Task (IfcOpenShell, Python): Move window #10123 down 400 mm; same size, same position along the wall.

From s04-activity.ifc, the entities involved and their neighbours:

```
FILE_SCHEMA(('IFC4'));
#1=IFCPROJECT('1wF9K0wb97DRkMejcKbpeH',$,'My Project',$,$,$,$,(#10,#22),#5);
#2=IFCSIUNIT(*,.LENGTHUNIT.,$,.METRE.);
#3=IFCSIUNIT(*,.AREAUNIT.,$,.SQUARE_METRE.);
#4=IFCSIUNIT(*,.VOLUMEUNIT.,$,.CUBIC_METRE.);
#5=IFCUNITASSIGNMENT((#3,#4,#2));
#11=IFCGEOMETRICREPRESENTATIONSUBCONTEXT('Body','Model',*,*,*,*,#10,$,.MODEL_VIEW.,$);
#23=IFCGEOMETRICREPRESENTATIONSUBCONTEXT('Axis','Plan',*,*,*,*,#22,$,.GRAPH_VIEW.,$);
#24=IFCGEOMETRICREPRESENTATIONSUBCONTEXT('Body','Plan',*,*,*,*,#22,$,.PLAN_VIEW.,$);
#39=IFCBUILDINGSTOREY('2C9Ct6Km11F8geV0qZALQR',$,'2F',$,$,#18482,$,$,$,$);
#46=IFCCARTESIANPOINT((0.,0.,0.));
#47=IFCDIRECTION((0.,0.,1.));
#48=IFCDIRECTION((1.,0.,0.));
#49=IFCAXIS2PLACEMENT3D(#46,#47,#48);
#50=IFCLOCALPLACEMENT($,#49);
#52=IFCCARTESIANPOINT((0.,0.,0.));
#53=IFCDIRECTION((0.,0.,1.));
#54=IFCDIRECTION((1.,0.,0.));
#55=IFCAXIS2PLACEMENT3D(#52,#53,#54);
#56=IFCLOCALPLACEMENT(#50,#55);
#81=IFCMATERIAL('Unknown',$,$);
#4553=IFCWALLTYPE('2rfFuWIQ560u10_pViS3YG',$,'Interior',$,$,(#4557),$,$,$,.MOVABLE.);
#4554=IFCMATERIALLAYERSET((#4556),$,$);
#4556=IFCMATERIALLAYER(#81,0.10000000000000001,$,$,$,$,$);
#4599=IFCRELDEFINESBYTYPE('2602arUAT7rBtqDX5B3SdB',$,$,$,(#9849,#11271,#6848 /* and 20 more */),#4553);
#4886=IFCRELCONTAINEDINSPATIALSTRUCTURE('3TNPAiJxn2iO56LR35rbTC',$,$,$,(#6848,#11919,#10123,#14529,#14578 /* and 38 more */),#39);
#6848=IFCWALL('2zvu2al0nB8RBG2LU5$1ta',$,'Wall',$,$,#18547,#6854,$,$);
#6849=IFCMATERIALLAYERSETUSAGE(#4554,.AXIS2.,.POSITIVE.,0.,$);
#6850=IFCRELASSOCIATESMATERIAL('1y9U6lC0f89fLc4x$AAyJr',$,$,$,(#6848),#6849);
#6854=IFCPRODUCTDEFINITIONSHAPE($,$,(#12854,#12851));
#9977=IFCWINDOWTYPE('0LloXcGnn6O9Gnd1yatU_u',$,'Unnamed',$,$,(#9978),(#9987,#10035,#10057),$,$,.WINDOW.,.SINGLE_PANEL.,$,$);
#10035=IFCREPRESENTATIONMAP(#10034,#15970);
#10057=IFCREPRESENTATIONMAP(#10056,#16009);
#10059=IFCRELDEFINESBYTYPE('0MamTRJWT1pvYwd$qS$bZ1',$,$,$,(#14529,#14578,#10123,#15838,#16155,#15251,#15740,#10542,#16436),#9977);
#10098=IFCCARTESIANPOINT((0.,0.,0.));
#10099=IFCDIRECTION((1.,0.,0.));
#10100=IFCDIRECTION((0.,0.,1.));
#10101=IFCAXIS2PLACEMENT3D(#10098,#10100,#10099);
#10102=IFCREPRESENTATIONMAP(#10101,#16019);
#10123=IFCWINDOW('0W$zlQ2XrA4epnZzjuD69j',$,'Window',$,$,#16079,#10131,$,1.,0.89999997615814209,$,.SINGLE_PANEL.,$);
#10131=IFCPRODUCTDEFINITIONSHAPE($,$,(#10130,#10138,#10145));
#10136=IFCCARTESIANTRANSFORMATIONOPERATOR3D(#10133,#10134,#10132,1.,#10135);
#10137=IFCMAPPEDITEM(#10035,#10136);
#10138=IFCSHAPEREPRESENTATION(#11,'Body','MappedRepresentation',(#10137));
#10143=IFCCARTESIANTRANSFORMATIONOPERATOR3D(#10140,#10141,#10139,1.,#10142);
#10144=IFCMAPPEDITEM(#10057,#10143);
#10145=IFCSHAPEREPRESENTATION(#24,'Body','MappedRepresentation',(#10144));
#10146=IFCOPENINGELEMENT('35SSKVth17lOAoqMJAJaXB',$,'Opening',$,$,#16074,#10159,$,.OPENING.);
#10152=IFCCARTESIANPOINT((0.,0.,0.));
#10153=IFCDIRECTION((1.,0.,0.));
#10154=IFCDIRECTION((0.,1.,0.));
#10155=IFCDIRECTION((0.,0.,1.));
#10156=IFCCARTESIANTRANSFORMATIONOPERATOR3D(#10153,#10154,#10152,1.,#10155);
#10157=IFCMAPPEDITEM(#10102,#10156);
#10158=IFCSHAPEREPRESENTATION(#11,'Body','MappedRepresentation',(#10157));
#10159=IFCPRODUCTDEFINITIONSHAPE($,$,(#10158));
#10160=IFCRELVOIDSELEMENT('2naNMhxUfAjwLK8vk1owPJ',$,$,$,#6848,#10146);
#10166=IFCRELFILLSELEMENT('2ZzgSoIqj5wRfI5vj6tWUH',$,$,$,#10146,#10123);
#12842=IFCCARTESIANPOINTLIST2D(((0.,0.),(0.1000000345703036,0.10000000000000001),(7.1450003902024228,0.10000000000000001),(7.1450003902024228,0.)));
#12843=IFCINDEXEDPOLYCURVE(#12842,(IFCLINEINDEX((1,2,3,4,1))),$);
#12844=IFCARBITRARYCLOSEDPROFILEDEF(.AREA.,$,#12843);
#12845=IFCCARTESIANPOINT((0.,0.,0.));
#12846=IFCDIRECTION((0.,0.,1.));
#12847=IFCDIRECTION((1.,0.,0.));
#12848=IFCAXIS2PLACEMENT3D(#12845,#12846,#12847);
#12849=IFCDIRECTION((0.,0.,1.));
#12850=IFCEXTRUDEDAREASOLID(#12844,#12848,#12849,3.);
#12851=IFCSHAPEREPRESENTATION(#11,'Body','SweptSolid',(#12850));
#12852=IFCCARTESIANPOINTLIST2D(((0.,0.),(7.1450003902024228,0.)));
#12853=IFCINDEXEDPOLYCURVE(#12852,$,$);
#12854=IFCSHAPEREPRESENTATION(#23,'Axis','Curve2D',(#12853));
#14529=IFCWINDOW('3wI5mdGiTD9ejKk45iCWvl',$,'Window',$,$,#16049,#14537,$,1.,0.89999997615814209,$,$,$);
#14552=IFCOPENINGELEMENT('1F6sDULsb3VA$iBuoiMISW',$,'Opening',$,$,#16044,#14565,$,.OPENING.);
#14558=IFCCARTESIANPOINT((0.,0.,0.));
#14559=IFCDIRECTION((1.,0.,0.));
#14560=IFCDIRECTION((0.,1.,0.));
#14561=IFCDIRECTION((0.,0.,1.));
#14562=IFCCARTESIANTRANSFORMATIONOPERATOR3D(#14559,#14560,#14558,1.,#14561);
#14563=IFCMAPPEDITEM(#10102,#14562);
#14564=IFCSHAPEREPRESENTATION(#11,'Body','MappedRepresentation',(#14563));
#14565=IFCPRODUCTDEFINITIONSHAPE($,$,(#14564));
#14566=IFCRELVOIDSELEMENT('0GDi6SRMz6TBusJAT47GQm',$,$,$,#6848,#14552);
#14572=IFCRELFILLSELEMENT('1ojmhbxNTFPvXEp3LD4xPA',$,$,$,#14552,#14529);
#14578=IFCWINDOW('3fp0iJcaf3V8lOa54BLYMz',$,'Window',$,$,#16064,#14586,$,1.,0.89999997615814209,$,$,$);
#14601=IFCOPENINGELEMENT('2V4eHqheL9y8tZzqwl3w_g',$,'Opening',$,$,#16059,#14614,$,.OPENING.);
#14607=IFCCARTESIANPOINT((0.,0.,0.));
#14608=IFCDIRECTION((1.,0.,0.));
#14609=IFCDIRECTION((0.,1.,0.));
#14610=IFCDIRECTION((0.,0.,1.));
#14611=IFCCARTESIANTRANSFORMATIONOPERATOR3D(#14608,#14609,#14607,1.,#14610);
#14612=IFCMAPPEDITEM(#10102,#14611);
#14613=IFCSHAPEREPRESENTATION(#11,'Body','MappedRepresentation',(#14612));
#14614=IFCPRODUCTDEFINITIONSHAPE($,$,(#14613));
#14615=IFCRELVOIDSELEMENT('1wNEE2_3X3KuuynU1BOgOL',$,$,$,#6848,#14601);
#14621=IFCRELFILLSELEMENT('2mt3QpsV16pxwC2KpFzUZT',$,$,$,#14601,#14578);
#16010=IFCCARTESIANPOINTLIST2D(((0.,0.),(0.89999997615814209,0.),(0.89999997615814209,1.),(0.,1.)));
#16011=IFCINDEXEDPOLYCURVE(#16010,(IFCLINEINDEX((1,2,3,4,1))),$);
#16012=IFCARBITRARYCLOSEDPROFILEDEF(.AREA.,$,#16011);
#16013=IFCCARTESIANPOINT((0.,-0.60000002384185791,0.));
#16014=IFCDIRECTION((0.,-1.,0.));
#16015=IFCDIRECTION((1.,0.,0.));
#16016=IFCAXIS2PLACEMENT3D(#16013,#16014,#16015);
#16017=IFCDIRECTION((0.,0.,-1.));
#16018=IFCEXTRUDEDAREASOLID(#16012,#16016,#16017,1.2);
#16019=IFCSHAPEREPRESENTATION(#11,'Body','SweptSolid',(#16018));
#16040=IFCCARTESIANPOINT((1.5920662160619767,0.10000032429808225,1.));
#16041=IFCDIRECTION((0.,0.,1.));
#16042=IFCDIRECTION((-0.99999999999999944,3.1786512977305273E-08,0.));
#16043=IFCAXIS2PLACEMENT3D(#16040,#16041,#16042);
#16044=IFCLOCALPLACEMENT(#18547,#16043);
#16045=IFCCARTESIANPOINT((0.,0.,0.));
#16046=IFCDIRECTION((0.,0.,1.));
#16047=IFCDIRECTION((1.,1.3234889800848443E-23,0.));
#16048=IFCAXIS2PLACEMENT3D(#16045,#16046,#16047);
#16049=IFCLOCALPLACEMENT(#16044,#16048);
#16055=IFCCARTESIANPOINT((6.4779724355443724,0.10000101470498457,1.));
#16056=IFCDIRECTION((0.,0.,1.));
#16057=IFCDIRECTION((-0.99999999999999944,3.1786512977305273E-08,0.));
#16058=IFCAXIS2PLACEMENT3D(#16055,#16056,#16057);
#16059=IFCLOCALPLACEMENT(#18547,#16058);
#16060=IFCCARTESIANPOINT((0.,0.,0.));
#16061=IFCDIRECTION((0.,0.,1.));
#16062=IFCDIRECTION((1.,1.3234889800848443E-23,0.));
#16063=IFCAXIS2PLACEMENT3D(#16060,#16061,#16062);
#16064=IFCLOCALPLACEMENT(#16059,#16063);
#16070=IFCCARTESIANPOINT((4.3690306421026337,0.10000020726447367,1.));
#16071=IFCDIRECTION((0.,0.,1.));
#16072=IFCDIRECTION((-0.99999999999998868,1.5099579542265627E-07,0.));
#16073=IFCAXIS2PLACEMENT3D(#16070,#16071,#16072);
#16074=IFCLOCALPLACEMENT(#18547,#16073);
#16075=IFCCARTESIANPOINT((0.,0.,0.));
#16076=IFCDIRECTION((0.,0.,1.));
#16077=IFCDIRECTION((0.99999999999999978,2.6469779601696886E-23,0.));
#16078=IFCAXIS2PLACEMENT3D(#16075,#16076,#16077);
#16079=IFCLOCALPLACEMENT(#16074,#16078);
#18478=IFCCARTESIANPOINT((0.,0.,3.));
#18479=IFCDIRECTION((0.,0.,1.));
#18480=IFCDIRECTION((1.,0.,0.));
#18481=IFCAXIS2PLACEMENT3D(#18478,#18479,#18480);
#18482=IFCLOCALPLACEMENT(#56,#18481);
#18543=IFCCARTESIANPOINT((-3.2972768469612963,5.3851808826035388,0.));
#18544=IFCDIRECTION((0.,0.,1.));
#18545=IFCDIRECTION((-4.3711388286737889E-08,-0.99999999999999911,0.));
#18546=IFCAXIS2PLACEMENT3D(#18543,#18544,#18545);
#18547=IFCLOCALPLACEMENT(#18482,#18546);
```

```python
import numpy as np
import ifcopenshell
import ifcopenshell.api.geometry
import ifcopenshell.util.placement
import ifcopenshell.util.unit

model = ifcopenshell.open("s04-activity.ifc")
unit_scale = ifcopenshell.util.unit.calculate_unit_scale(model)

window = model.by_guid("0W$zlQ2XrA4epnZzjuD69j")
opening = window.FillsVoids[0].RelatingOpeningElement
dz = -0.4 / unit_scale

shift = np.array([0.0, 0.0, dz])
# The window is placed relative to its opening, so it follows when the opening moves.
matrix = ifcopenshell.util.placement.get_local_placement(opening.ObjectPlacement)
matrix[:3, 3] += shift
ifcopenshell.api.geometry.edit_object_placement(
    model, product=opening, matrix=matrix, is_si=False, should_transform_children=True
)

print(f"moved by {dz * unit_scale:+.3f} m")

model.write("s04-activity_rev.ifc")
```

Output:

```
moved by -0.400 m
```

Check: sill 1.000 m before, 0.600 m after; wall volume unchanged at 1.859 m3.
